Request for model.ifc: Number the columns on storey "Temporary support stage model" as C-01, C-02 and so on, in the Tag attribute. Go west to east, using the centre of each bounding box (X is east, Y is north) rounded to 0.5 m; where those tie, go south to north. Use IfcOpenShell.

First a look at what the model holds.

```python
import ifcopenshell
import ifcopenshell.util.element
import ifcopenshell.util.placement

model = ifcopenshell.open("model.ifc")
print(model.schema)
storey = next(s for s in model.by_type("IfcBuildingStorey") if s.Name == "Temporary support stage model")
columns = [e for e in ifcopenshell.util.element.get_decomposition(storey) if e.is_a("IfcColumn")]
for e in sorted(columns, key=lambda e: e.id()):
    origin = ifcopenshell.util.placement.get_local_placement(e.ObjectPlacement)[:3, 3]
    print(e.id(), e.Tag, e.Name, origin.round(2) + 0.0, sep=" | ")
```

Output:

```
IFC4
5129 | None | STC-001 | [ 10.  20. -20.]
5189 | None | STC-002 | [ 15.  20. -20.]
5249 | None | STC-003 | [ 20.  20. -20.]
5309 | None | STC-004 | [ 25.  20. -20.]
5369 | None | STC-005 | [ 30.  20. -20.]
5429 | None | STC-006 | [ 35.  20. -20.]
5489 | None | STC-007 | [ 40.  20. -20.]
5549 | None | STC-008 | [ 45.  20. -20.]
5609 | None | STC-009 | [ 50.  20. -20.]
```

```python
import ifcopenshell
import ifcopenshell.geom
import ifcopenshell.util.element
import ifcopenshell.util.shape

model = ifcopenshell.open("model.ifc")
settings = ifcopenshell.geom.settings()
settings.set("use-world-coords", True)


def centre(element):
    shape = ifcopenshell.geom.create_shape(settings, element)
    return ifcopenshell.util.shape.get_bbox_centroid(shape.geometry)


storey = next(s for s in model.by_type("IfcBuildingStorey") if s.Name == "Temporary support stage model")
columns = [e for e in ifcopenshell.util.element.get_decomposition(storey) if e.is_a("IfcColumn")]

# Insertion points can sit at a corner or the storey origin, so sort by the geometry (in metres).
centres = {e: centre(e) for e in columns}
columns.sort(key=lambda e: (round(centres[e][0] / 0.5), centres[e][1]))

for i, e in enumerate(columns, start=1):
    number = f"C-{i:02d}"
    e.Tag = number
    print(e.id(), number)

model.write("model_updated.ifc")
```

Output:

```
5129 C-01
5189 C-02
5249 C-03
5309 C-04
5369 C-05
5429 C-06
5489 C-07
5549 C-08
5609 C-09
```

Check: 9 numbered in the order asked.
